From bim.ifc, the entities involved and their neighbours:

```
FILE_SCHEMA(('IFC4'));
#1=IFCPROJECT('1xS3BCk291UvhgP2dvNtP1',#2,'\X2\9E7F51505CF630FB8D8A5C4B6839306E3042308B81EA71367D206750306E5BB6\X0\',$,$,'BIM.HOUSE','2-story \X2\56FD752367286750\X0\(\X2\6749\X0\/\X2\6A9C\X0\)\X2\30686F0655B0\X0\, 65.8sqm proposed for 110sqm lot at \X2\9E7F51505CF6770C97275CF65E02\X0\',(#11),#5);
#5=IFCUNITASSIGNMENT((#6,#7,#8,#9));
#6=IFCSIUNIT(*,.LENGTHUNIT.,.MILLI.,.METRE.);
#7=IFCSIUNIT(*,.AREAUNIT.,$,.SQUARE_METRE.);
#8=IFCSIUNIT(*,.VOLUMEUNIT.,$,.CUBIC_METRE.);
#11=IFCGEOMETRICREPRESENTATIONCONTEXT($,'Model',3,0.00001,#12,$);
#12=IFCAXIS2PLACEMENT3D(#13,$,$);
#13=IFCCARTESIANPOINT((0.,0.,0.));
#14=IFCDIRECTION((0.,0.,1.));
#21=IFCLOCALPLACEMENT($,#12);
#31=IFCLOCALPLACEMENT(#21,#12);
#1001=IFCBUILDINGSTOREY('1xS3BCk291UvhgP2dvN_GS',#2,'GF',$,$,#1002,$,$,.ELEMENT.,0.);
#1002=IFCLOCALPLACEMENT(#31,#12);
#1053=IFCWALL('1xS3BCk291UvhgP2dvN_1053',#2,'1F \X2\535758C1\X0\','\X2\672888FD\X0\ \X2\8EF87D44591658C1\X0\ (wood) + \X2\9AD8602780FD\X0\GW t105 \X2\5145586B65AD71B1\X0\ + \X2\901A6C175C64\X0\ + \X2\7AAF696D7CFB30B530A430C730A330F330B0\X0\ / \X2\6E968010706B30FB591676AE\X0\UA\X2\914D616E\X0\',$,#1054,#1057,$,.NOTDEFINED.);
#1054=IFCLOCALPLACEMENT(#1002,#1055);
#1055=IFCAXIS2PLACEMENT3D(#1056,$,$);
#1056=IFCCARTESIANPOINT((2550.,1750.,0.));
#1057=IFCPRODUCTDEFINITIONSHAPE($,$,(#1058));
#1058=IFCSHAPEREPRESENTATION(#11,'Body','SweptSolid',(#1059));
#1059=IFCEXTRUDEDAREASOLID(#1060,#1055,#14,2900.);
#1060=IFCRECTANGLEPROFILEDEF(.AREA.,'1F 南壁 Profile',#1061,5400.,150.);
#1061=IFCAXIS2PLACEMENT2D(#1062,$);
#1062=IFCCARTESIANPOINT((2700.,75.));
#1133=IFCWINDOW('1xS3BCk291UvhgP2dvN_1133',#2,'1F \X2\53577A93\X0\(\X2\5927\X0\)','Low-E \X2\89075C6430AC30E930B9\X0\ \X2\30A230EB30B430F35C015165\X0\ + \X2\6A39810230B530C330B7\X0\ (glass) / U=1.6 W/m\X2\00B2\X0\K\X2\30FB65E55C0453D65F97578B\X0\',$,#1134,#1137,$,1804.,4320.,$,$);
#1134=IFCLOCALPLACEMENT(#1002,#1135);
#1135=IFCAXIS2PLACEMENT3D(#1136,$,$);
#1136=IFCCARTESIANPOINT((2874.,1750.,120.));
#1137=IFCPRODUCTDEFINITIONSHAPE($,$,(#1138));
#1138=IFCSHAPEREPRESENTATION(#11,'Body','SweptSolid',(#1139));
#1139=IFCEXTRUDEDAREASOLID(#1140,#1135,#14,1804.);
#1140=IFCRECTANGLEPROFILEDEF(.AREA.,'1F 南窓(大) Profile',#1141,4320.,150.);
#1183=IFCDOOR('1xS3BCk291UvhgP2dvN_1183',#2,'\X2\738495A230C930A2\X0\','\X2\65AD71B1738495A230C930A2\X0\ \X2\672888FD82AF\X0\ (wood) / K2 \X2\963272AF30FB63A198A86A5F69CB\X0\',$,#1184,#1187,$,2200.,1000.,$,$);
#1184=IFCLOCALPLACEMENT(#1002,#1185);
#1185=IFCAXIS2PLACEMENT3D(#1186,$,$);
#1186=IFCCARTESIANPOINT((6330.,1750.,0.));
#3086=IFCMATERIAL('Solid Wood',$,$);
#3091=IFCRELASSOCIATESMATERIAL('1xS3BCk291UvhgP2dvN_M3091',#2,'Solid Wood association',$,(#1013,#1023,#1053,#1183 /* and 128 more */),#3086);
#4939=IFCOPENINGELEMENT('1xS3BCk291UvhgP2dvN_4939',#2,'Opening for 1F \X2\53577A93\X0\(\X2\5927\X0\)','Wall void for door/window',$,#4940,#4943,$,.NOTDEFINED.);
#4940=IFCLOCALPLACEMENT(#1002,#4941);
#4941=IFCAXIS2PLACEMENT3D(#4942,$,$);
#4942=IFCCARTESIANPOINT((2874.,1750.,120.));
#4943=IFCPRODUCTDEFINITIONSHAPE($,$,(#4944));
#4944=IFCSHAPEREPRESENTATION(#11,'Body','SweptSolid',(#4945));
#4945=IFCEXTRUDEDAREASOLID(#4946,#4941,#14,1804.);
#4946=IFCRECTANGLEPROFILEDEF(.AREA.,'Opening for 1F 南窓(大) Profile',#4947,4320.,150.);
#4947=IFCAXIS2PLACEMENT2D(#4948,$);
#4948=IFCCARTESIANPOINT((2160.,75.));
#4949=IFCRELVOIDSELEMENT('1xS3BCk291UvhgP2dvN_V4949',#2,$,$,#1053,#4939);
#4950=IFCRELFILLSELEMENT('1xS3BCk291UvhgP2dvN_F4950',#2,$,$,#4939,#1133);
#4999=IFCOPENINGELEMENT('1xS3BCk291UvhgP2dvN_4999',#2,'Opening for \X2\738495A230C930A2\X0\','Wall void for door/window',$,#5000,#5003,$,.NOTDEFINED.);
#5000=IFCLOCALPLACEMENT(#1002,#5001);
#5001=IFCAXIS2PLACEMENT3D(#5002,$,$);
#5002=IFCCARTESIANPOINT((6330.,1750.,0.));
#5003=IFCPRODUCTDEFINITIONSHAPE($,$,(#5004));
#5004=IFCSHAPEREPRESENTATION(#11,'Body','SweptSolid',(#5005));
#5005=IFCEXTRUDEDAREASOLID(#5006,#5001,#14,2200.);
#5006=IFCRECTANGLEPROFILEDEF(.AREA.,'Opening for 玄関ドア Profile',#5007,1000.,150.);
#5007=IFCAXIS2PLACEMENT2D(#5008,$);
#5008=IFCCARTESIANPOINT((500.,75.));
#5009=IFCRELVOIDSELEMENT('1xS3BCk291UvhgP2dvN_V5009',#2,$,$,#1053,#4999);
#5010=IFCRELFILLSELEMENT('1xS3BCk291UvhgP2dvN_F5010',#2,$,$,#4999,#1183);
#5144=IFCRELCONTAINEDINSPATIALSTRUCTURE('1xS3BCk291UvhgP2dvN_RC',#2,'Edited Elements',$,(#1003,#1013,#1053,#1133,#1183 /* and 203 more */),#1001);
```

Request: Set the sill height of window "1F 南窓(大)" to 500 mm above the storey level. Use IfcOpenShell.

```python
import numpy as np
import ifcopenshell
import ifcopenshell.api.geometry
import ifcopenshell.geom
import ifcopenshell.util.element
import ifcopenshell.util.placement
import ifcopenshell.util.shape
import ifcopenshell.util.unit

model = ifcopenshell.open("bim.ifc")
unit_scale = ifcopenshell.util.unit.calculate_unit_scale(model)

window = model.by_guid("1xS3BCk291UvhgP2dvN_1133")
opening = window.FillsVoids[0].RelatingOpeningElement
storey = ifcopenshell.util.element.get_container(window, ifc_class="IfcBuildingStorey")
level = ifcopenshell.util.placement.get_local_placement(storey.ObjectPlacement)[2, 3]

# The opening's origin need not be at the sill, so measure its lowest point.
shape = ifcopenshell.geom.create_shape(ifcopenshell.geom.settings(), opening)
bottom = ifcopenshell.util.shape.get_shape_bottom_elevation(shape, shape.geometry) / unit_scale
dz = level + 0.5 / unit_scale - bottom

shift = np.array([0.0, 0.0, dz])
# The window is not placed relative to its opening, so move both.
for product in (opening, window):
    matrix = ifcopenshell.util.placement.get_local_placement(product.ObjectPlacement)
    matrix[:3, 3] += shift
    ifcopenshell.api.geometry.edit_object_placement(model, product=product, matrix=matrix, is_si=False)

print(f"moved by {dz * unit_scale:+.3f} m")

model.write("bim-out.ifc")
```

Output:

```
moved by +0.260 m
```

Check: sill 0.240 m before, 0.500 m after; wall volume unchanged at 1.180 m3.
